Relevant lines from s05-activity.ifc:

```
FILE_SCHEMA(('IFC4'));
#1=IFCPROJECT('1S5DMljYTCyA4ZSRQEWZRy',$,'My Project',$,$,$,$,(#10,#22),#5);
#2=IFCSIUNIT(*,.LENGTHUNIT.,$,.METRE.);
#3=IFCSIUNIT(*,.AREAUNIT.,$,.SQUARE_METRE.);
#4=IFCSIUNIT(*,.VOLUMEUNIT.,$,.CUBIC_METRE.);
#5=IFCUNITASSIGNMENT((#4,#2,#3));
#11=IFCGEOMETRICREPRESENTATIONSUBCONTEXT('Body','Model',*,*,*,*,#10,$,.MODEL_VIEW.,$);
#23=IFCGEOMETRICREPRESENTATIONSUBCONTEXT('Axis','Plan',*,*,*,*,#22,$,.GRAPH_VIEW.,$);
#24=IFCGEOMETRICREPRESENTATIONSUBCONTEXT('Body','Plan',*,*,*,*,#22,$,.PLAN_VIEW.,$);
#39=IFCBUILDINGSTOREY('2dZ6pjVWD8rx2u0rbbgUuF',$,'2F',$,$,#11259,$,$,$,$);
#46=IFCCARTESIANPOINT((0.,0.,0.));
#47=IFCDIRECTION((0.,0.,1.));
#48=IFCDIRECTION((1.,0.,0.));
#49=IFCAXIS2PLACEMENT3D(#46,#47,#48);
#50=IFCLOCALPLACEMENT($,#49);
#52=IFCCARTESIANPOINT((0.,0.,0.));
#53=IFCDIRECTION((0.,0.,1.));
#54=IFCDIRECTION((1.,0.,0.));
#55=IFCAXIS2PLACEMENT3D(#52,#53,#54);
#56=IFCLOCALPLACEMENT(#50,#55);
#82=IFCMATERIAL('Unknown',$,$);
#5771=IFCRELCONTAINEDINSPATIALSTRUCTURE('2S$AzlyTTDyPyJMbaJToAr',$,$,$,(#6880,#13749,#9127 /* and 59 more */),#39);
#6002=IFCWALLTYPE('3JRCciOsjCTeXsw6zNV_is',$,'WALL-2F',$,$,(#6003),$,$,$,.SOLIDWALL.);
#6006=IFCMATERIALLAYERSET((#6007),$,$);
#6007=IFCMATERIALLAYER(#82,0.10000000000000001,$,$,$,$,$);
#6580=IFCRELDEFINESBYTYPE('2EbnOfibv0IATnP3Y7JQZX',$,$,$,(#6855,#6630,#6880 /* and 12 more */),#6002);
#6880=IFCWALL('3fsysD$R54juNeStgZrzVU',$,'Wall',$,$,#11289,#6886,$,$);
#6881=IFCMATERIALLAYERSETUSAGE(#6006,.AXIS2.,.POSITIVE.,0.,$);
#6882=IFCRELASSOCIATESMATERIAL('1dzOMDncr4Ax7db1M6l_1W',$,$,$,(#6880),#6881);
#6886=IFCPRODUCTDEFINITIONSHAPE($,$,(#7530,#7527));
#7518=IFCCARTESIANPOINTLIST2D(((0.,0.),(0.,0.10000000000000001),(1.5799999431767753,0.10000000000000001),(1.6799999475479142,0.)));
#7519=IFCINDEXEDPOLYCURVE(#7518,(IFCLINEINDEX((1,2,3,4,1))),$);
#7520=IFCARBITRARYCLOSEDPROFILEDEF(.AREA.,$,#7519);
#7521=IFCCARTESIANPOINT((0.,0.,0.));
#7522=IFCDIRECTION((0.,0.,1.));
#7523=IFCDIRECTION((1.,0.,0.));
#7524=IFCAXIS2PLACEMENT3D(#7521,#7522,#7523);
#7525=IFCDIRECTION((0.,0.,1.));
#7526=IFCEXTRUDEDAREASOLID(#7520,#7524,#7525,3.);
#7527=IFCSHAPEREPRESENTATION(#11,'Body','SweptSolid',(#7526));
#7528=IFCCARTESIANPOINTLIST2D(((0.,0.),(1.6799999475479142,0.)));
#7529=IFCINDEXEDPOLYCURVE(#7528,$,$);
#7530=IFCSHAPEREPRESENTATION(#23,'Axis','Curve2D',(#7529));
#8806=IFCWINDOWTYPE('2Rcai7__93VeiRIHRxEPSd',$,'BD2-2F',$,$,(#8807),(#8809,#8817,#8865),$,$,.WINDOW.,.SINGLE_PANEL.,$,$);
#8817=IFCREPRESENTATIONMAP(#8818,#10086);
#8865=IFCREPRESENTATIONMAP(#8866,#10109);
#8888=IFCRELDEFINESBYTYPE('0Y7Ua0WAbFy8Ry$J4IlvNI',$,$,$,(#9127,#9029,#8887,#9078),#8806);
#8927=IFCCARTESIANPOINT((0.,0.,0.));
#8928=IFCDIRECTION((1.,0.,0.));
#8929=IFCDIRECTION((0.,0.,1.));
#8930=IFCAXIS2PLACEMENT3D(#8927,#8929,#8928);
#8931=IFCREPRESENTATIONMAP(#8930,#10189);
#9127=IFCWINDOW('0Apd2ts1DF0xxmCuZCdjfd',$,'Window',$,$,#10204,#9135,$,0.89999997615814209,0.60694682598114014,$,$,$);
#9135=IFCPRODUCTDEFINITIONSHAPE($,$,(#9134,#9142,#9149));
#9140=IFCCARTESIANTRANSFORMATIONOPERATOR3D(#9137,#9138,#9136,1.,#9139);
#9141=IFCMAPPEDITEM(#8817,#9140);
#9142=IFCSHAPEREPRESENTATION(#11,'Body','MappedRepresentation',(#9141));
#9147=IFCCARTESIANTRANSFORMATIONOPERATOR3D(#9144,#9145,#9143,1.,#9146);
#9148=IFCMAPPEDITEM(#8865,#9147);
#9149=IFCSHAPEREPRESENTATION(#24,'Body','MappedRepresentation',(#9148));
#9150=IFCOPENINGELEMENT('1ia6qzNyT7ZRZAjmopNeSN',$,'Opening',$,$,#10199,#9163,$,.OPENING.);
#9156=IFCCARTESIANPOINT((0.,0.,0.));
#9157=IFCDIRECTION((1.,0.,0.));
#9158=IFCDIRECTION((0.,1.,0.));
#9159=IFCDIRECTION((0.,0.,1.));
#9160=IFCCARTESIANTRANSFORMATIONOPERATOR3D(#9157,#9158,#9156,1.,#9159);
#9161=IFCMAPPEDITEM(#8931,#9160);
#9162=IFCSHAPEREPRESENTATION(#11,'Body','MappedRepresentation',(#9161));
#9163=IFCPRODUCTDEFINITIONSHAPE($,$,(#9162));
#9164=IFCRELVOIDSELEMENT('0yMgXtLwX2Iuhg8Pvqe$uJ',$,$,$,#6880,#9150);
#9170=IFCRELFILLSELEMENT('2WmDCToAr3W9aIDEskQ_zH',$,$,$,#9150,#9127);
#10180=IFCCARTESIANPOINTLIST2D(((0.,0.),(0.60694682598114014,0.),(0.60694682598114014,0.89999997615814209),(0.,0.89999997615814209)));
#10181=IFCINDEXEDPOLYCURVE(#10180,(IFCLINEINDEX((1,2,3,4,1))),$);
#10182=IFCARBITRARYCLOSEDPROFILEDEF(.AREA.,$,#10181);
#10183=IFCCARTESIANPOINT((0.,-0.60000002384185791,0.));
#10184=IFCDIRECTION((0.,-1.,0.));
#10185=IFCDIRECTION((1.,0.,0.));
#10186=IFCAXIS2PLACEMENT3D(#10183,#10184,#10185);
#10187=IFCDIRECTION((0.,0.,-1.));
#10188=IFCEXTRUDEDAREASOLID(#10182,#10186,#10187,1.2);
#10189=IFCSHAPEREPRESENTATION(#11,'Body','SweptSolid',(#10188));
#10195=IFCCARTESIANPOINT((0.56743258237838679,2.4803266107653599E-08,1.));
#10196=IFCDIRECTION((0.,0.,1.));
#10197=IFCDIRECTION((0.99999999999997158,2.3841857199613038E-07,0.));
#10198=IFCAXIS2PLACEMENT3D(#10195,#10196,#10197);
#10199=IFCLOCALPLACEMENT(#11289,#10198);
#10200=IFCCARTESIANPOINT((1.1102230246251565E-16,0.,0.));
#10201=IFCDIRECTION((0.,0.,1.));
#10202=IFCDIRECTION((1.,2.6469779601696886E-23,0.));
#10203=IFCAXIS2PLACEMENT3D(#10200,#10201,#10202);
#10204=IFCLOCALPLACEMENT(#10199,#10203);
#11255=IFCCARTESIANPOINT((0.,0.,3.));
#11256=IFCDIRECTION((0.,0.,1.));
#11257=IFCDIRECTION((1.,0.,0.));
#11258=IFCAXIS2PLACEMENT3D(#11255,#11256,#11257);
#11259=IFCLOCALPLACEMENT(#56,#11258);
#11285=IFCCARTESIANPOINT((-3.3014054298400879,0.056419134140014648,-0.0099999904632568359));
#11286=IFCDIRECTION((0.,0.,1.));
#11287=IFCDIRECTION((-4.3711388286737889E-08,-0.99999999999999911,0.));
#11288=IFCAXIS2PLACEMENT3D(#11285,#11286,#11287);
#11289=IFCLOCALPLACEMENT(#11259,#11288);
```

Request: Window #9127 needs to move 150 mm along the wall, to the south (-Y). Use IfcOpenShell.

```python
import ifcopenshell
import ifcopenshell.api.geometry
import ifcopenshell.util.placement
import ifcopenshell.util.unit

model = ifcopenshell.open("s05-activity.ifc")
unit_scale = ifcopenshell.util.unit.calculate_unit_scale(model)

window = model.by_id(9127)
opening = window.FillsVoids[0].RelatingOpeningElement
wall = opening.VoidsElements[0].RelatingBuildingElement

wall_matrix = ifcopenshell.util.placement.get_local_placement(wall.ObjectPlacement)
shift = wall_matrix[:3, 0] * 0.15 / unit_scale
before = ifcopenshell.util.placement.get_local_placement(window.ObjectPlacement)[:3, 3].copy()

# The window is placed relative to its opening, so it follows when the opening moves.
matrix = ifcopenshell.util.placement.get_local_placement(opening.ObjectPlacement)
matrix[:3, 3] += shift
ifcopenshell.api.geometry.edit_object_placement(
    model, product=opening, matrix=matrix, is_si=False, should_transform_children=True
)

after = ifcopenshell.util.placement.get_local_placement(window.ObjectPlacement)[:3, 3]
print("window moved by", (after - before).round(3) + 0.0)

model.write("s05-activity_edited.ifc")
```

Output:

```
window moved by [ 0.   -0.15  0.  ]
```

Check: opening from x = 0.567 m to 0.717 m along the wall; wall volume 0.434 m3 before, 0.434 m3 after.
